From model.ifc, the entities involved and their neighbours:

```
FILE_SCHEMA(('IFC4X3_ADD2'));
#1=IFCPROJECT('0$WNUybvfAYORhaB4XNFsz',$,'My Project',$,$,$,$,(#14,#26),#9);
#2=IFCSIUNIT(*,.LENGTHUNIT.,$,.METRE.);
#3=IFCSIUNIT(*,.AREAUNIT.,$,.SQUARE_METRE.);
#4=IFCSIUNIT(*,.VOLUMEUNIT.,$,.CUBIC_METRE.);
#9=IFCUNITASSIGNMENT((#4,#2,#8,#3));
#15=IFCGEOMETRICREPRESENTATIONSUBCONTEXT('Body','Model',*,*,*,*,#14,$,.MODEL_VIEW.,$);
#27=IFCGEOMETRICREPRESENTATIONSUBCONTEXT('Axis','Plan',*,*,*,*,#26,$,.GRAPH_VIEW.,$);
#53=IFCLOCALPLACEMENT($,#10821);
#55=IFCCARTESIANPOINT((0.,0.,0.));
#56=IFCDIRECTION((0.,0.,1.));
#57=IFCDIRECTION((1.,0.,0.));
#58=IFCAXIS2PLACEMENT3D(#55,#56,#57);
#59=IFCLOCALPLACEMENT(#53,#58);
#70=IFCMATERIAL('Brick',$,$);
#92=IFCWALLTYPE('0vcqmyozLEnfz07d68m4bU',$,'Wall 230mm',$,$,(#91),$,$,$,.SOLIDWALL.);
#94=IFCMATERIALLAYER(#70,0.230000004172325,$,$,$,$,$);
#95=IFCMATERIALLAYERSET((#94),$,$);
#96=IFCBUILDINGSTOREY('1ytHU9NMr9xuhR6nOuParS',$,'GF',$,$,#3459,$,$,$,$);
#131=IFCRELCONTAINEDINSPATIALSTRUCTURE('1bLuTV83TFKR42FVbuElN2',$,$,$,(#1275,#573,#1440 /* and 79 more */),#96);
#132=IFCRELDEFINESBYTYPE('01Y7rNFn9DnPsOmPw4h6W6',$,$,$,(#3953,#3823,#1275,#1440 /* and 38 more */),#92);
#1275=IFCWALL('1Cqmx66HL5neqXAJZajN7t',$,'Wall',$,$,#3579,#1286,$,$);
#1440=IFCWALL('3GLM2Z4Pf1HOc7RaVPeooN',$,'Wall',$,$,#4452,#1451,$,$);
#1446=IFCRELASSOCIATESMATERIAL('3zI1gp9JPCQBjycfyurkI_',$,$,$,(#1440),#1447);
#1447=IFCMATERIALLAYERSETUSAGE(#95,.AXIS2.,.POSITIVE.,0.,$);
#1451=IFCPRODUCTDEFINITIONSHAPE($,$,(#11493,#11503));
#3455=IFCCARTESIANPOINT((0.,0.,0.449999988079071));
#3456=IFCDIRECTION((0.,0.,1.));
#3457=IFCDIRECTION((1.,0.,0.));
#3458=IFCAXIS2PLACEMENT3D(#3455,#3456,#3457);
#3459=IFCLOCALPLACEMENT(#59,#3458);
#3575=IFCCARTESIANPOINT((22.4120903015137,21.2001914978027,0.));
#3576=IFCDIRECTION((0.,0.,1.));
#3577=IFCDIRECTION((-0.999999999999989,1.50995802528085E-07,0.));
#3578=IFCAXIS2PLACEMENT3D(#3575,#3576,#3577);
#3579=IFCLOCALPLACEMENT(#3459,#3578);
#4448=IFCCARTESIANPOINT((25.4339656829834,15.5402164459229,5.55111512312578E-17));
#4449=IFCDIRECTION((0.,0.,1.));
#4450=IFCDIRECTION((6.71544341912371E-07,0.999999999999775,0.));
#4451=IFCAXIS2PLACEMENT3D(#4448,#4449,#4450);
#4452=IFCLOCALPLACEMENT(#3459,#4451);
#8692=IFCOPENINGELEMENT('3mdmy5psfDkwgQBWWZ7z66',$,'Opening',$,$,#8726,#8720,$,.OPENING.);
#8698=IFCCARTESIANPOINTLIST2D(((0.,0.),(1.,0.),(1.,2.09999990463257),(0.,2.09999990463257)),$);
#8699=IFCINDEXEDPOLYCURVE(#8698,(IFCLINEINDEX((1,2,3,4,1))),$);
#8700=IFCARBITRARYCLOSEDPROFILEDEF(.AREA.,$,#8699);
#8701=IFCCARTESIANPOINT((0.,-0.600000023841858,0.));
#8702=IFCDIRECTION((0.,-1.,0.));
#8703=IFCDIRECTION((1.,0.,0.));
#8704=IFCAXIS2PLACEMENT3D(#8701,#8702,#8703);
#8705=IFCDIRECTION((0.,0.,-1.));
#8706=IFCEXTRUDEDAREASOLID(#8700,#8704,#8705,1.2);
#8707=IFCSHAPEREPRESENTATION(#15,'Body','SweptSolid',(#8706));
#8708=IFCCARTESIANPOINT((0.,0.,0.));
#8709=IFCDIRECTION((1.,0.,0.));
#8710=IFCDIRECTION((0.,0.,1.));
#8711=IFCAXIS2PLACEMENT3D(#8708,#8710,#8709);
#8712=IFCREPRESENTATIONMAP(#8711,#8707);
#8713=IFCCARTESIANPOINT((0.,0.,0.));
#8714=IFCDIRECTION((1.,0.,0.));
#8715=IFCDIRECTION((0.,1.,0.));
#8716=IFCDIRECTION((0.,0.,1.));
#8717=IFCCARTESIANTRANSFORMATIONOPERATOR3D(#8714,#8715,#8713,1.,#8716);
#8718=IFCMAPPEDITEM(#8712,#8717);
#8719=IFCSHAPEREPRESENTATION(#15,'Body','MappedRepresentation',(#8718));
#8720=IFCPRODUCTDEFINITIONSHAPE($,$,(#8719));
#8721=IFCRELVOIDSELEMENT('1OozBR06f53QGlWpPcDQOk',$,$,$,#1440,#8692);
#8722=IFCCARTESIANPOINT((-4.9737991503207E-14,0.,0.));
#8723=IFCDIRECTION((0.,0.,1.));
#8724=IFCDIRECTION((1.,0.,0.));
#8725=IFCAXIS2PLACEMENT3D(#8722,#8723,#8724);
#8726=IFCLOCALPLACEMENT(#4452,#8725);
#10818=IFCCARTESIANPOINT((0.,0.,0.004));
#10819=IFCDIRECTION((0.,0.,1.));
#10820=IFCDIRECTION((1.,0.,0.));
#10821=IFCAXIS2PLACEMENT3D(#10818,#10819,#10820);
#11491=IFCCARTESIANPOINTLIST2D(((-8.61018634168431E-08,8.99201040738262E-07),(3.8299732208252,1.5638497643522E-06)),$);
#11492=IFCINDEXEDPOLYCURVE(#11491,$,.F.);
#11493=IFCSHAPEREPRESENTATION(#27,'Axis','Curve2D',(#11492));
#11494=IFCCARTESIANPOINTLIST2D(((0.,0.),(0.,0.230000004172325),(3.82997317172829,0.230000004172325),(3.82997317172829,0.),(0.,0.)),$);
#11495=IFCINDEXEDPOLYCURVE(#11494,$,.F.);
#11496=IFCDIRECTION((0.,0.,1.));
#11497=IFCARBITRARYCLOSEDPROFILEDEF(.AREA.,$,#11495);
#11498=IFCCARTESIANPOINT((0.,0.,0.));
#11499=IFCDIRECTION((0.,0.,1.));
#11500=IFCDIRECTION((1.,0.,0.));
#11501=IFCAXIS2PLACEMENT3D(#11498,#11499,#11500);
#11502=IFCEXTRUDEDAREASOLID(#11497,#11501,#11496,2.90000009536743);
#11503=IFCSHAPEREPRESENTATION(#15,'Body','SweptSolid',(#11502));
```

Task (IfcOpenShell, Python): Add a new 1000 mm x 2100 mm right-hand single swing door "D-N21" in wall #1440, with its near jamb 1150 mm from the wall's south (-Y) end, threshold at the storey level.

```python
import numpy as np
import ifcopenshell
import ifcopenshell.api.feature
import ifcopenshell.api.geometry
import ifcopenshell.api.root
import ifcopenshell.api.spatial
import ifcopenshell.geom
import ifcopenshell.util.element
import ifcopenshell.util.placement
import ifcopenshell.util.representation
import ifcopenshell.util.shape
import ifcopenshell.util.unit

model = ifcopenshell.open("model.ifc")
unit_scale = ifcopenshell.util.unit.calculate_unit_scale(model)
settings = ifcopenshell.geom.settings()


def volume(element):
    """Net volume in cubic metres, openings subtracted."""
    shape = ifcopenshell.geom.create_shape(settings, element)
    return ifcopenshell.util.shape.get_volume(shape.geometry)


wall = model.by_guid("3GLM2Z4Pf1HOc7RaVPeooN")
storey = ifcopenshell.util.element.get_container(wall, ifc_class="IfcBuildingStorey")
context = ifcopenshell.util.representation.get_context(model, "Model", "Body", "MODEL_VIEW")
before = volume(wall)

width, height, from_end, sill = 1, 2.1, 1.15, 0.0  # metres

# The wall runs along its own X axis, and the end named is its -X end.
wall_shape = ifcopenshell.geom.create_shape(settings, wall)
x, y, z = ifcopenshell.util.shape.get_vertices(wall_shape.geometry).T
start = x.min() + from_end
face, thickness = float(y.min()), float(y.max() - y.min())
wall_matrix = ifcopenshell.util.placement.get_local_placement(wall.ObjectPlacement)
level = ifcopenshell.util.placement.get_local_placement(storey.ObjectPlacement)[2, 3]


def in_wall(x, y):
    """Placement at x, y metres in the wall's axes, at sill height."""
    matrix = wall_matrix.copy()
    matrix[:, 3] = wall_matrix @ np.array([x / unit_scale, y / unit_scale, 0.0, 1.0])
    matrix[2, 3] = level + sill / unit_scale
    return matrix


# Opening: a box that overshoots both wall faces by 50 mm.
opening = ifcopenshell.api.root.create_entity(model, ifc_class="IfcOpeningElement", predefined_type="OPENING")
box = ifcopenshell.api.geometry.add_wall_representation(
    model, context=context, length=width, height=height, thickness=thickness + 0.1
)
ifcopenshell.api.geometry.assign_representation(model, product=opening, representation=box)
ifcopenshell.api.geometry.edit_object_placement(model, product=opening, matrix=in_wall(start, face - 0.05), is_si=False)
ifcopenshell.api.feature.add_feature(model, feature=opening, element=wall)

door = ifcopenshell.api.root.create_entity(model, ifc_class="IfcDoor", name="D-N21", predefined_type="DOOR")
door.OverallWidth, door.OverallHeight = width / unit_scale, height / unit_scale
door.OperationType = "SINGLE_SWING_RIGHT"
body = ifcopenshell.api.geometry.add_door_representation(
    model,
    context=context,
    overall_width=door.OverallWidth,
    overall_height=door.OverallHeight,
    operation_type="SINGLE_SWING_RIGHT",
    lining_properties={"LiningDepth": thickness / unit_scale, "ThresholdDepth": thickness / unit_scale},
)
ifcopenshell.api.geometry.assign_representation(model, product=door, representation=body)
ifcopenshell.api.spatial.assign_container(model, products=[door], relating_structure=storey)
ifcopenshell.api.feature.add_filling(model, opening=opening, element=door)

# The lining spans the wall, so the door starts at the wall face.
ifcopenshell.api.geometry.edit_object_placement(model, product=door, matrix=in_wall(start, face), is_si=False)

after = volume(wall)

print(f"wall volume {before:.3f} -> {after:.3f} m3")

model.write("model-out.ifc")
```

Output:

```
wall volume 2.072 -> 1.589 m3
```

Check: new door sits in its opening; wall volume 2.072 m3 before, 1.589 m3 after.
